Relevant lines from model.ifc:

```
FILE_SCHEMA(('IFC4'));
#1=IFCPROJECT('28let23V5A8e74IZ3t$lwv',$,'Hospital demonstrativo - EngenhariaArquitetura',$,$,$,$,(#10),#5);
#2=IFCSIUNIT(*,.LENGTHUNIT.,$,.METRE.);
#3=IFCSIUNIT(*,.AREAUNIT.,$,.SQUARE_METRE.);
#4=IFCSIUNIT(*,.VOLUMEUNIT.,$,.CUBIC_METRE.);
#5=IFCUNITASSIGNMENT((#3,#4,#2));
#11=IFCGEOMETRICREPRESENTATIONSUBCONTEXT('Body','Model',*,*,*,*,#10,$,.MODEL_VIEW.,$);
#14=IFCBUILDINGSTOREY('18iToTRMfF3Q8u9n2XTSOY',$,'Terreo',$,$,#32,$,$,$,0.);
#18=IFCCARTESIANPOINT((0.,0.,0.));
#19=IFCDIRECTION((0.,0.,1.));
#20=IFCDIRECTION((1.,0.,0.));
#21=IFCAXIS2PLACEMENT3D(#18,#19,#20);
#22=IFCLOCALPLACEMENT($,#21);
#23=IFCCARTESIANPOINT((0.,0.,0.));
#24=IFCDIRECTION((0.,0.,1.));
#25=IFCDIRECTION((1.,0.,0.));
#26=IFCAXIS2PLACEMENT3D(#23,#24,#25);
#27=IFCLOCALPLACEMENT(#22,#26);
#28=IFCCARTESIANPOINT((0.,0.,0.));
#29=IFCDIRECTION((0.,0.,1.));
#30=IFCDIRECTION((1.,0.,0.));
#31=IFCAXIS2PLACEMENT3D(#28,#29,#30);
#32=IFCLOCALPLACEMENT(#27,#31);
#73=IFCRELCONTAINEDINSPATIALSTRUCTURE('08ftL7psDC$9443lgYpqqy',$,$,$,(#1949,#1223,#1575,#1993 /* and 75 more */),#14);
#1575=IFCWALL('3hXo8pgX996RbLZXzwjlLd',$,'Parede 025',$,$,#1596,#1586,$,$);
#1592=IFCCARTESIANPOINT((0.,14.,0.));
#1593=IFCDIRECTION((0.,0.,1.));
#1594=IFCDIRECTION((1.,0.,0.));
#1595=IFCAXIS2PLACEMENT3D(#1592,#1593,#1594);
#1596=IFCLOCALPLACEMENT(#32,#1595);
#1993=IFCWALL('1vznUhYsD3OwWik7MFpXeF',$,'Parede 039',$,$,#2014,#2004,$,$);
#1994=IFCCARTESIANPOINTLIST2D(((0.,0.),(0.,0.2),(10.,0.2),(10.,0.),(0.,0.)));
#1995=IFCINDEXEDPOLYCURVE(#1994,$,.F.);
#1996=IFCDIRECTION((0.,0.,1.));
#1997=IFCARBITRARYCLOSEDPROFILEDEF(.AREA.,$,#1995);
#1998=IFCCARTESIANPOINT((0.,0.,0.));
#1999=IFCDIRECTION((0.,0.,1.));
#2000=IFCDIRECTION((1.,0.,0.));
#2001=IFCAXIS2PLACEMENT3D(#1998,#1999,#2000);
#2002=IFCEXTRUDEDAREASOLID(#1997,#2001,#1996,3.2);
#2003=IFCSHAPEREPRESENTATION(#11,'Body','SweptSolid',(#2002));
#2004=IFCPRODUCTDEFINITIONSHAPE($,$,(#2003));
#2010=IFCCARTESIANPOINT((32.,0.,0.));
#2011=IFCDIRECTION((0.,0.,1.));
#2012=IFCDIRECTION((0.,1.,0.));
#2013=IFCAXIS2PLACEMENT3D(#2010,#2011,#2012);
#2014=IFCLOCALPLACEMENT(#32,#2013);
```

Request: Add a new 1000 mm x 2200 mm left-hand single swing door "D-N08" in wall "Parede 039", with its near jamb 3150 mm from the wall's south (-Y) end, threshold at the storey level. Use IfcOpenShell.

```python
import numpy as np
import ifcopenshell
import ifcopenshell.api.feature
import ifcopenshell.api.geometry
import ifcopenshell.api.root
import ifcopenshell.api.spatial
import ifcopenshell.geom
import ifcopenshell.util.element
import ifcopenshell.util.placement
import ifcopenshell.util.representation
import ifcopenshell.util.shape
import ifcopenshell.util.unit

model = ifcopenshell.open("model.ifc")
unit_scale = ifcopenshell.util.unit.calculate_unit_scale(model)
settings = ifcopenshell.geom.settings()


def volume(element):
    """Net volume in cubic metres, openings subtracted."""
    shape = ifcopenshell.geom.create_shape(settings, element)
    return ifcopenshell.util.shape.get_volume(shape.geometry)


wall = model.by_id(1993)
storey = ifcopenshell.util.element.get_container(wall, ifc_class="IfcBuildingStorey")
context = ifcopenshell.util.representation.get_context(model, "Model", "Body", "MODEL_VIEW")
before = volume(wall)

width, height, from_end, sill = 1, 2.2, 3.15, 0.0  # metres

# The wall runs along its own X axis, and the end named is its -X end.
wall_shape = ifcopenshell.geom.create_shape(settings, wall)
x, y, z = ifcopenshell.util.shape.get_vertices(wall_shape.geometry).T
start = x.min() + from_end
face, thickness = float(y.min()), float(y.max() - y.min())
wall_matrix = ifcopenshell.util.placement.get_local_placement(wall.ObjectPlacement)
level = ifcopenshell.util.placement.get_local_placement(storey.ObjectPlacement)[2, 3]


def in_wall(x, y):
    """Placement at x, y metres in the wall's axes, at sill height."""
    matrix = wall_matrix.copy()
    matrix[:, 3] = wall_matrix @ np.array([x / unit_scale, y / unit_scale, 0.0, 1.0])
    matrix[2, 3] = level + sill / unit_scale
    return matrix


# Opening: a box that overshoots both wall faces by 50 mm.
opening = ifcopenshell.api.root.create_entity(model, ifc_class="IfcOpeningElement", predefined_type="OPENING")
box = ifcopenshell.api.geometry.add_wall_representation(
    model, context=context, length=width, height=height, thickness=thickness + 0.1
)
ifcopenshell.api.geometry.assign_representation(model, product=opening, representation=box)
ifcopenshell.api.geometry.edit_object_placement(model, product=opening, matrix=in_wall(start, face - 0.05), is_si=False)
ifcopenshell.api.feature.add_feature(model, feature=opening, element=wall)

door = ifcopenshell.api.root.create_entity(model, ifc_class="IfcDoor", name="D-N08", predefined_type="DOOR")
door.OverallWidth, door.OverallHeight = width / unit_scale, height / unit_scale
door.OperationType = "SINGLE_SWING_LEFT"
body = ifcopenshell.api.geometry.add_door_representation(
    model,
    context=context,
    overall_width=door.OverallWidth,
    overall_height=door.OverallHeight,
    operation_type="SINGLE_SWING_LEFT",
    lining_properties={"LiningDepth": thickness / unit_scale, "ThresholdDepth": thickness / unit_scale},
)
ifcopenshell.api.geometry.assign_representation(model, product=door, representation=body)
ifcopenshell.api.spatial.assign_container(model, products=[door], relating_structure=storey)
ifcopenshell.api.feature.add_filling(model, opening=opening, element=door)

# The lining spans the wall, so the door starts at the wall face.
ifcopenshell.api.geometry.edit_object_placement(model, product=door, matrix=in_wall(start, face), is_si=False)

after = volume(wall)

print(f"wall volume {before:.3f} -> {after:.3f} m3")

model.write("model-out.ifc")
```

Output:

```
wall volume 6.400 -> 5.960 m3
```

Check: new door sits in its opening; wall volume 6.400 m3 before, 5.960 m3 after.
